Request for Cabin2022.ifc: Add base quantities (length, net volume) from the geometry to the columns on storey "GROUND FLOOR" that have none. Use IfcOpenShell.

First a look at what the model holds.

```python
import ifcopenshell
import ifcopenshell.util.element
import ifcopenshell.util.unit

model = ifcopenshell.open("Cabin2022.ifc")
print(model.schema)
for unit_type in ("LENGTHUNIT", "AREAUNIT", "VOLUMEUNIT"):
    print(unit_type, ifcopenshell.util.unit.calculate_unit_scale(model, unit_type))
storey = next(s for s in model.by_type("IfcBuildingStorey") if s.Name == "GROUND FLOOR")
columns = [e for e in ifcopenshell.util.element.get_decomposition(storey) if e.is_a("IfcColumn")]
for e in sorted(columns, key=lambda e: e.id()):
    print(e.id(), e.is_a(), e.Name, list(ifcopenshell.util.element.get_psets(e, qtos_only=True)), sep=" | ")
```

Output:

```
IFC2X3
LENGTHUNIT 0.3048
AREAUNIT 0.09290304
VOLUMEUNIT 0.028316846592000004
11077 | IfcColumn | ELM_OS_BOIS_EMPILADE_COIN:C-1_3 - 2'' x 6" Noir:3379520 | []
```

```python
import ifcopenshell
import ifcopenshell.api.pset
import ifcopenshell.geom
import ifcopenshell.util.element
import ifcopenshell.util.shape
import ifcopenshell.util.unit

model = ifcopenshell.open("Cabin2022.ifc")
unit_scale = ifcopenshell.util.unit.calculate_unit_scale(model)
volume_scale = ifcopenshell.util.unit.calculate_unit_scale(model, "VOLUMEUNIT")
settings = ifcopenshell.geom.settings()

storey = next(s for s in model.by_type("IfcBuildingStorey") if s.Name == "GROUND FLOOR")
columns = [e for e in ifcopenshell.util.element.get_decomposition(storey) if e.is_a("IfcColumn")]

for e in sorted(columns, key=lambda e: e.id()):
    if ifcopenshell.util.element.get_psets(e, qtos_only=True, should_inherit=False):
        continue
    # Geometry comes back in metres, in the element's own axes.
    shape = ifcopenshell.geom.create_shape(settings, e)
    values = {
        "Length": ifcopenshell.util.shape.get_z(shape.geometry) / unit_scale,
        "NetVolume": ifcopenshell.util.shape.get_volume(shape.geometry) / volume_scale,
    }
    qto = ifcopenshell.api.pset.add_qto(model, product=e, name="BaseQuantities")
    ifcopenshell.api.pset.edit_qto(model, qto=qto, properties=values)
    print(e.id(), {k: round(v, 3) for k, v in values.items()})

model.write("Cabin2022_rev.ifc")
```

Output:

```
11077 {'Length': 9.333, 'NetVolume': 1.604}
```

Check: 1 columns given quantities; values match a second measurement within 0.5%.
